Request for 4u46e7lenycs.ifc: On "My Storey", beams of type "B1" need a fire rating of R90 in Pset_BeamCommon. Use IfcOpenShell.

First a look at what the model holds.

```python
import ifcopenshell
import ifcopenshell.util.element

model = ifcopenshell.open("4u46e7lenycs.ifc")
print(model.schema)
storey = next(s for s in model.by_type("IfcBuildingStorey") if s.Name == "My Storey")
beams = [e for e in ifcopenshell.util.element.get_decomposition(storey) if e.is_a("IfcBeam")]
seen = {}
for e in beams:
    element_type = ifcopenshell.util.element.get_type(e)
    key = (element_type.Name if element_type != e and element_type else None, ifcopenshell.util.element.get_pset(e, "Pset_BeamCommon", "FireRating"))
    seen[key] = seen.get(key, 0) + 1
for (name, value), count in sorted(seen.items(), key=str):
    print(count, "x", name, "|", value)
```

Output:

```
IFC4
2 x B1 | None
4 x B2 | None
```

```python
import ifcopenshell
import ifcopenshell.api.pset
import ifcopenshell.util.element

model = ifcopenshell.open("4u46e7lenycs.ifc")

storey = next(s for s in model.by_type("IfcBuildingStorey") if s.Name == "My Storey")
beams = [e for e in ifcopenshell.util.element.get_decomposition(storey) if e.is_a("IfcBeam")]

count = 0
for e in beams:
    element_type = ifcopenshell.util.element.get_type(e)
    if element_type in (None, e) or element_type.Name != "B1":
        continue
    # add_pset returns the element's existing set when there is one.
    pset = ifcopenshell.api.pset.add_pset(model, product=e, name="Pset_BeamCommon")
    ifcopenshell.api.pset.edit_pset(model, pset=pset, properties={"FireRating": "R90"})
    count += 1

print(count, "beams updated")

model.write("4u46e7lenycs_rev.ifc")
```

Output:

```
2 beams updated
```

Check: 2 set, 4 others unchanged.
